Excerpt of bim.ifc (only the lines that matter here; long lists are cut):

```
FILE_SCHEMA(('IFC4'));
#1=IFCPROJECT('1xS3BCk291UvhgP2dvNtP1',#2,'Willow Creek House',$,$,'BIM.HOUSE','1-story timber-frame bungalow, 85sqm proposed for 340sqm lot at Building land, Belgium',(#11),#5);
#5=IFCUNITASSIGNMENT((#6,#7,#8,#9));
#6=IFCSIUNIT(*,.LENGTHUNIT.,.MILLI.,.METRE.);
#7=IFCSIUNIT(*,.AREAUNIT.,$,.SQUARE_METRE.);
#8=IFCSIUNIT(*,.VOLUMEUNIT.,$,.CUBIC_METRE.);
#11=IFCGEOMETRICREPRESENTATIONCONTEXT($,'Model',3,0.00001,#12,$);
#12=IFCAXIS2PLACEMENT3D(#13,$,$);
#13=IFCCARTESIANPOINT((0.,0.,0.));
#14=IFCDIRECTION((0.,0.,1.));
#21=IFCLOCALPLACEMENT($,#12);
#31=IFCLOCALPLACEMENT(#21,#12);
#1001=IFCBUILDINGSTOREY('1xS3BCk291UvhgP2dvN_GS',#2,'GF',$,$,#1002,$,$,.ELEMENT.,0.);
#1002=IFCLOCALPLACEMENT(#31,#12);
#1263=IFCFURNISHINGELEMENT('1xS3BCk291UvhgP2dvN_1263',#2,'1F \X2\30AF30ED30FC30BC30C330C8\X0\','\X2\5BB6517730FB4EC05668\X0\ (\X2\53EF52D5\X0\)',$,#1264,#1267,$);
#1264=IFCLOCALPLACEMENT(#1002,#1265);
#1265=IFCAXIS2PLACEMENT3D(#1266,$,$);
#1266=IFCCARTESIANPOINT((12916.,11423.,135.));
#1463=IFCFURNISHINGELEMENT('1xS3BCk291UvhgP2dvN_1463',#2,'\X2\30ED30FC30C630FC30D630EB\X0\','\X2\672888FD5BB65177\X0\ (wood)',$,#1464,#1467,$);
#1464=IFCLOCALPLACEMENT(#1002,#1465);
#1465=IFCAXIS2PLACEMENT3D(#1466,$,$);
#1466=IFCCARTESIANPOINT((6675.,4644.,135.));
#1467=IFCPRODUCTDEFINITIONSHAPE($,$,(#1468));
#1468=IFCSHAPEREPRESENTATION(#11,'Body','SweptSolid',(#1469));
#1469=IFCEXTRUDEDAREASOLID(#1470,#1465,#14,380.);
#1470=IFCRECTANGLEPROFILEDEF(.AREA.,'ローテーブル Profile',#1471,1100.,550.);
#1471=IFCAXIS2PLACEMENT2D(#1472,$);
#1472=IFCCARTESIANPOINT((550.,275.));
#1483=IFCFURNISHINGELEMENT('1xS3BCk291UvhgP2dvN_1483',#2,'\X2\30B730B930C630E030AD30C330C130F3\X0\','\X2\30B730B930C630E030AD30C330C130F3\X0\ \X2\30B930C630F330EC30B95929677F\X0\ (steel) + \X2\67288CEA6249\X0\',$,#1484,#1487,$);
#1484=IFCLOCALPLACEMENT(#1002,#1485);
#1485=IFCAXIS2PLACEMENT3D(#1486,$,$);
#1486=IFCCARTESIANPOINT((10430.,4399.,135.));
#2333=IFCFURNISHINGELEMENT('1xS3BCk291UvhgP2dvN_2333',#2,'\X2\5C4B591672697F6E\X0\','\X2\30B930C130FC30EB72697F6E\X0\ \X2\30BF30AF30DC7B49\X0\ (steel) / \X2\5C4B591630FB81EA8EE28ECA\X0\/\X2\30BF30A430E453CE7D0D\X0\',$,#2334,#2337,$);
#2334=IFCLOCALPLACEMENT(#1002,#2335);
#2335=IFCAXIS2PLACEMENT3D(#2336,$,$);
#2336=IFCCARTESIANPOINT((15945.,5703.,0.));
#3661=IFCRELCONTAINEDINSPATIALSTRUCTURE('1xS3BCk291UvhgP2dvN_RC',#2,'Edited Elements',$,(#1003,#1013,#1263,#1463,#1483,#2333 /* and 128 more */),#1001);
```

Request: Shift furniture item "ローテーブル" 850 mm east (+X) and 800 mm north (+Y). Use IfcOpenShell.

```python
import ifcopenshell
import ifcopenshell.api.geometry
import ifcopenshell.util.placement
import ifcopenshell.util.unit

model = ifcopenshell.open("bim.ifc")
unit_scale = ifcopenshell.util.unit.calculate_unit_scale(model)

item = model.by_id(1463)
matrix = ifcopenshell.util.placement.get_local_placement(item.ObjectPlacement)
matrix[0, 3] += 0.85 / unit_scale
matrix[1, 3] += 0.8 / unit_scale
ifcopenshell.api.geometry.edit_object_placement(model, product=item, matrix=matrix, is_si=False)

print(ifcopenshell.util.placement.get_local_placement(item.ObjectPlacement).round(3) + 0.0)

model.write("bim_rev.ifc")
```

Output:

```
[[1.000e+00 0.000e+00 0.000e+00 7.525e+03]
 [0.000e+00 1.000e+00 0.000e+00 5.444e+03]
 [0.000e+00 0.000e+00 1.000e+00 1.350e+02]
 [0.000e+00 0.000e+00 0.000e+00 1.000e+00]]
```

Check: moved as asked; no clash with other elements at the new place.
